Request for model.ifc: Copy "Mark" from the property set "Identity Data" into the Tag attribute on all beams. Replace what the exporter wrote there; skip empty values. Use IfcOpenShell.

First a look at what the model holds.

```python
import ifcopenshell
import ifcopenshell.util.element

model = ifcopenshell.open("model.ifc")
print(model.schema)
beams = model.by_type("IfcBeam")
print(len(beams), "beams")
for e in beams[:8]:
    source = ifcopenshell.util.element.get_pset(e, "Identity Data", "Mark")
    target = e.Tag
    print(e.id(), repr(source), repr(target), sep=" | ")
```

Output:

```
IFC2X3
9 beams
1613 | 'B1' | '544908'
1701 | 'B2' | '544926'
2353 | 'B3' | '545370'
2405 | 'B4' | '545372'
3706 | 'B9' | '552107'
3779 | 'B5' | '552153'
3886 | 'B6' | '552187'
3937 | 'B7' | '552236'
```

```python
import ifcopenshell
import ifcopenshell.util.element

model = ifcopenshell.open("model.ifc")

count = 0
for e in model.by_type("IfcBeam"):
    value = ifcopenshell.util.element.get_pset(e, "Identity Data", "Mark")
    current = e.Tag
    if not value or not value.strip() or current == value:
        continue
    e.Tag = value
    count += 1

print(count, "beams updated")

model.write("model_v2.ifc")
```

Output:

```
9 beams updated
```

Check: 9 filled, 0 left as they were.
